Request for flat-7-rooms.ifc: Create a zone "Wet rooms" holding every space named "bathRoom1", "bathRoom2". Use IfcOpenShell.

First a look at what the model holds.

```python
import ifcopenshell

model = ifcopenshell.open("flat-7-rooms.ifc")
print(model.schema)
seen = {}
for space in model.by_type("IfcSpace"):
    seen[space.LongName] = seen.get(space.LongName, 0) + 1
for name, count in sorted(seen.items(), key=str):
    print(count, "x", name)
print("zones:", [z.Name for z in model.by_type("IfcZone")][:20])
```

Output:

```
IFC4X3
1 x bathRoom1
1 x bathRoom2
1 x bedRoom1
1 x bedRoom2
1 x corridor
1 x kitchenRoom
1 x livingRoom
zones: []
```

```python
import ifcopenshell
import ifcopenshell.api.group
import ifcopenshell.api.root

model = ifcopenshell.open("flat-7-rooms.ifc")

names = {"bathRoom1", "bathRoom2"}
spaces = [s for s in model.by_type("IfcSpace") if s.LongName in names]

zone = ifcopenshell.api.root.create_entity(model, ifc_class="IfcZone", name="Wet rooms")
ifcopenshell.api.group.assign_group(model, products=spaces, group=zone)
print(len(spaces), "spaces in", zone.Name)

model.write("flat-7-rooms_updated.ifc")
```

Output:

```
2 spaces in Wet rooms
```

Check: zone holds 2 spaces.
